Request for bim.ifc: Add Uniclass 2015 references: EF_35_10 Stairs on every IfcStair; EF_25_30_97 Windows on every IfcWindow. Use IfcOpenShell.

First a look at what the model holds.

```python
import ifcopenshell

model = ifcopenshell.open("bim.ifc")
print(model.schema)
print("classifications:", [c.Name for c in model.by_type("IfcClassification")])
for ifc_class in ("IfcDoor", "IfcRoof", "IfcStair", "IfcWall", "IfcWindow"):
    print(ifc_class, len(model.by_type(ifc_class)))
```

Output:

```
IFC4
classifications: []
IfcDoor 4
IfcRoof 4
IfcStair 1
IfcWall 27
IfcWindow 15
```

```python
import ifcopenshell
import ifcopenshell.api.classification

model = ifcopenshell.open("bim.ifc")

system = ifcopenshell.api.classification.add_classification(model, classification="Uniclass 2015")

codes = {
    "IfcStair": ("EF_35_10", "Stairs"),
    "IfcWindow": ("EF_25_30_97", "Windows"),
}
for ifc_class, (code, name) in codes.items():
    products = model.by_type(ifc_class)
    ifcopenshell.api.classification.add_reference(
        model, products=products, classification=system, identification=code, name=name
    )
    print(code, len(products))

model.write("bim-out.ifc")
```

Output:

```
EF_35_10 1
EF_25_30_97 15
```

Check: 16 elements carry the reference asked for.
